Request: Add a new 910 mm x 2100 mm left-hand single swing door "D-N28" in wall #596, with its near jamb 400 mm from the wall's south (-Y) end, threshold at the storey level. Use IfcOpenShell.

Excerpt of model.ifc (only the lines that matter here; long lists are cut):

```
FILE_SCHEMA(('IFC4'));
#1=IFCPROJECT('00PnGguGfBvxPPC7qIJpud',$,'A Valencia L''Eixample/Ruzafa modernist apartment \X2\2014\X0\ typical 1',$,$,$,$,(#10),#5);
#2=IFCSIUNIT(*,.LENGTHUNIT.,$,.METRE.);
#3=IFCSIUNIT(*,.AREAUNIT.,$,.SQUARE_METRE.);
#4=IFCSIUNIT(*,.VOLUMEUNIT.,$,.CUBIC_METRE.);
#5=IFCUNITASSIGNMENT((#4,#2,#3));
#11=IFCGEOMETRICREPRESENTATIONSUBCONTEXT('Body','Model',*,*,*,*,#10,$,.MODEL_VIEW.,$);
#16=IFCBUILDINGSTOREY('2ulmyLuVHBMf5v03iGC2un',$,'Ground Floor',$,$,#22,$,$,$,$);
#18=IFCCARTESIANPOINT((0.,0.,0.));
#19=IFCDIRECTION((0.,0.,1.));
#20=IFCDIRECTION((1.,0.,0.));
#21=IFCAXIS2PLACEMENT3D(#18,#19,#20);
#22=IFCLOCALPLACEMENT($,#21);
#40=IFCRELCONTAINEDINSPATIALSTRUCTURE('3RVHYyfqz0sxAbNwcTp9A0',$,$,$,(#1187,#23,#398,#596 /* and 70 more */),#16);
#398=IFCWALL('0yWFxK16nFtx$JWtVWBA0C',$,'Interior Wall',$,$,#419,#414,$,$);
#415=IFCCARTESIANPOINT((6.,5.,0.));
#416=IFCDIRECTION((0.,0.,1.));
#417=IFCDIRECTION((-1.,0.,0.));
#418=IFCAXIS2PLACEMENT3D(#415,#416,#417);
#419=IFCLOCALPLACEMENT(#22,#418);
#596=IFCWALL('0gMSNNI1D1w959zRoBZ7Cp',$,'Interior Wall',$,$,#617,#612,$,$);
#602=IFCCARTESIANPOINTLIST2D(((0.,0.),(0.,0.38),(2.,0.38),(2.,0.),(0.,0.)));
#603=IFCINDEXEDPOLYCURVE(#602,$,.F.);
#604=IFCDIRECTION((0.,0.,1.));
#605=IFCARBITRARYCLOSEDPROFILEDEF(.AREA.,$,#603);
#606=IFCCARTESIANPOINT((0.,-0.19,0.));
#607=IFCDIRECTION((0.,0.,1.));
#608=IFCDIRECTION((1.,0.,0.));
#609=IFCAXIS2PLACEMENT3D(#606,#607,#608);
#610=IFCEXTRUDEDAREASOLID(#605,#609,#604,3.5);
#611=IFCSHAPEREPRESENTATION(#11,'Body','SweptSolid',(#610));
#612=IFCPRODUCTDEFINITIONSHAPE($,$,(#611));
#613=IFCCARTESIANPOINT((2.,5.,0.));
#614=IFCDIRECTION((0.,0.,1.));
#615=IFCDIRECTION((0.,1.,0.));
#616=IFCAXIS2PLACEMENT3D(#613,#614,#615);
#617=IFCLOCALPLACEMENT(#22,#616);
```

```python
import numpy as np
import ifcopenshell
import ifcopenshell.api.feature
import ifcopenshell.api.geometry
import ifcopenshell.api.root
import ifcopenshell.api.spatial
import ifcopenshell.geom
import ifcopenshell.util.element
import ifcopenshell.util.placement
import ifcopenshell.util.representation
import ifcopenshell.util.shape
import ifcopenshell.util.unit

model = ifcopenshell.open("model.ifc")
unit_scale = ifcopenshell.util.unit.calculate_unit_scale(model)
settings = ifcopenshell.geom.settings()


def volume(element):
    """Net volume in cubic metres, openings subtracted."""
    shape = ifcopenshell.geom.create_shape(settings, element)
    return ifcopenshell.util.shape.get_volume(shape.geometry)


wall = model.by_guid("0gMSNNI1D1w959zRoBZ7Cp")
storey = ifcopenshell.util.element.get_container(wall, ifc_class="IfcBuildingStorey")
context = ifcopenshell.util.representation.get_context(model, "Model", "Body", "MODEL_VIEW")
before = volume(wall)

width, height, from_end, sill = 0.91, 2.1, 0.4, 0.0  # metres

# The wall runs along its own X axis, and the end named is its -X end.
wall_shape = ifcopenshell.geom.create_shape(settings, wall)
x, y, z = ifcopenshell.util.shape.get_vertices(wall_shape.geometry).T
start = x.min() + from_end
face, thickness = float(y.min()), float(y.max() - y.min())
wall_matrix = ifcopenshell.util.placement.get_local_placement(wall.ObjectPlacement)
level = ifcopenshell.util.placement.get_local_placement(storey.ObjectPlacement)[2, 3]


def in_wall(x, y):
    """Placement at x, y metres in the wall's axes, at sill height."""
    matrix = wall_matrix.copy()
    matrix[:, 3] = wall_matrix @ np.array([x / unit_scale, y / unit_scale, 0.0, 1.0])
    matrix[2, 3] = level + sill / unit_scale
    return matrix


# Opening: a box that overshoots both wall faces by 50 mm.
opening = ifcopenshell.api.root.create_entity(model, ifc_class="IfcOpeningElement", predefined_type="OPENING")
box = ifcopenshell.api.geometry.add_wall_representation(
    model, context=context, length=width, height=height, thickness=thickness + 0.1
)
ifcopenshell.api.geometry.assign_representation(model, product=opening, representation=box)
ifcopenshell.api.geometry.edit_object_placement(model, product=opening, matrix=in_wall(start, face - 0.05), is_si=False)
ifcopenshell.api.feature.add_feature(model, feature=opening, element=wall)

door = ifcopenshell.api.root.create_entity(model, ifc_class="IfcDoor", name="D-N28", predefined_type="DOOR")
door.OverallWidth, door.OverallHeight = width / unit_scale, height / unit_scale
door.OperationType = "SINGLE_SWING_LEFT"
body = ifcopenshell.api.geometry.add_door_representation(
    model,
    context=context,
    overall_width=door.OverallWidth,
    overall_height=door.OverallHeight,
    operation_type="SINGLE_SWING_LEFT",
    lining_properties={"LiningDepth": thickness / unit_scale, "ThresholdDepth": thickness / unit_scale},
)
ifcopenshell.api.geometry.assign_representation(model, product=door, representation=body)
ifcopenshell.api.spatial.assign_container(model, products=[door], relating_structure=storey)
ifcopenshell.api.feature.add_filling(model, opening=opening, element=door)

# The lining spans the wall, so the door starts at the wall face.
ifcopenshell.api.geometry.edit_object_placement(model, product=door, matrix=in_wall(start, face), is_si=False)

after = volume(wall)

print(f"wall volume {before:.3f} -> {after:.3f} m3")

model.write("model_rev.ifc")
```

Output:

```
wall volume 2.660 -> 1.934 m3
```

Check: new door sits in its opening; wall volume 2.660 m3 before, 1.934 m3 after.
